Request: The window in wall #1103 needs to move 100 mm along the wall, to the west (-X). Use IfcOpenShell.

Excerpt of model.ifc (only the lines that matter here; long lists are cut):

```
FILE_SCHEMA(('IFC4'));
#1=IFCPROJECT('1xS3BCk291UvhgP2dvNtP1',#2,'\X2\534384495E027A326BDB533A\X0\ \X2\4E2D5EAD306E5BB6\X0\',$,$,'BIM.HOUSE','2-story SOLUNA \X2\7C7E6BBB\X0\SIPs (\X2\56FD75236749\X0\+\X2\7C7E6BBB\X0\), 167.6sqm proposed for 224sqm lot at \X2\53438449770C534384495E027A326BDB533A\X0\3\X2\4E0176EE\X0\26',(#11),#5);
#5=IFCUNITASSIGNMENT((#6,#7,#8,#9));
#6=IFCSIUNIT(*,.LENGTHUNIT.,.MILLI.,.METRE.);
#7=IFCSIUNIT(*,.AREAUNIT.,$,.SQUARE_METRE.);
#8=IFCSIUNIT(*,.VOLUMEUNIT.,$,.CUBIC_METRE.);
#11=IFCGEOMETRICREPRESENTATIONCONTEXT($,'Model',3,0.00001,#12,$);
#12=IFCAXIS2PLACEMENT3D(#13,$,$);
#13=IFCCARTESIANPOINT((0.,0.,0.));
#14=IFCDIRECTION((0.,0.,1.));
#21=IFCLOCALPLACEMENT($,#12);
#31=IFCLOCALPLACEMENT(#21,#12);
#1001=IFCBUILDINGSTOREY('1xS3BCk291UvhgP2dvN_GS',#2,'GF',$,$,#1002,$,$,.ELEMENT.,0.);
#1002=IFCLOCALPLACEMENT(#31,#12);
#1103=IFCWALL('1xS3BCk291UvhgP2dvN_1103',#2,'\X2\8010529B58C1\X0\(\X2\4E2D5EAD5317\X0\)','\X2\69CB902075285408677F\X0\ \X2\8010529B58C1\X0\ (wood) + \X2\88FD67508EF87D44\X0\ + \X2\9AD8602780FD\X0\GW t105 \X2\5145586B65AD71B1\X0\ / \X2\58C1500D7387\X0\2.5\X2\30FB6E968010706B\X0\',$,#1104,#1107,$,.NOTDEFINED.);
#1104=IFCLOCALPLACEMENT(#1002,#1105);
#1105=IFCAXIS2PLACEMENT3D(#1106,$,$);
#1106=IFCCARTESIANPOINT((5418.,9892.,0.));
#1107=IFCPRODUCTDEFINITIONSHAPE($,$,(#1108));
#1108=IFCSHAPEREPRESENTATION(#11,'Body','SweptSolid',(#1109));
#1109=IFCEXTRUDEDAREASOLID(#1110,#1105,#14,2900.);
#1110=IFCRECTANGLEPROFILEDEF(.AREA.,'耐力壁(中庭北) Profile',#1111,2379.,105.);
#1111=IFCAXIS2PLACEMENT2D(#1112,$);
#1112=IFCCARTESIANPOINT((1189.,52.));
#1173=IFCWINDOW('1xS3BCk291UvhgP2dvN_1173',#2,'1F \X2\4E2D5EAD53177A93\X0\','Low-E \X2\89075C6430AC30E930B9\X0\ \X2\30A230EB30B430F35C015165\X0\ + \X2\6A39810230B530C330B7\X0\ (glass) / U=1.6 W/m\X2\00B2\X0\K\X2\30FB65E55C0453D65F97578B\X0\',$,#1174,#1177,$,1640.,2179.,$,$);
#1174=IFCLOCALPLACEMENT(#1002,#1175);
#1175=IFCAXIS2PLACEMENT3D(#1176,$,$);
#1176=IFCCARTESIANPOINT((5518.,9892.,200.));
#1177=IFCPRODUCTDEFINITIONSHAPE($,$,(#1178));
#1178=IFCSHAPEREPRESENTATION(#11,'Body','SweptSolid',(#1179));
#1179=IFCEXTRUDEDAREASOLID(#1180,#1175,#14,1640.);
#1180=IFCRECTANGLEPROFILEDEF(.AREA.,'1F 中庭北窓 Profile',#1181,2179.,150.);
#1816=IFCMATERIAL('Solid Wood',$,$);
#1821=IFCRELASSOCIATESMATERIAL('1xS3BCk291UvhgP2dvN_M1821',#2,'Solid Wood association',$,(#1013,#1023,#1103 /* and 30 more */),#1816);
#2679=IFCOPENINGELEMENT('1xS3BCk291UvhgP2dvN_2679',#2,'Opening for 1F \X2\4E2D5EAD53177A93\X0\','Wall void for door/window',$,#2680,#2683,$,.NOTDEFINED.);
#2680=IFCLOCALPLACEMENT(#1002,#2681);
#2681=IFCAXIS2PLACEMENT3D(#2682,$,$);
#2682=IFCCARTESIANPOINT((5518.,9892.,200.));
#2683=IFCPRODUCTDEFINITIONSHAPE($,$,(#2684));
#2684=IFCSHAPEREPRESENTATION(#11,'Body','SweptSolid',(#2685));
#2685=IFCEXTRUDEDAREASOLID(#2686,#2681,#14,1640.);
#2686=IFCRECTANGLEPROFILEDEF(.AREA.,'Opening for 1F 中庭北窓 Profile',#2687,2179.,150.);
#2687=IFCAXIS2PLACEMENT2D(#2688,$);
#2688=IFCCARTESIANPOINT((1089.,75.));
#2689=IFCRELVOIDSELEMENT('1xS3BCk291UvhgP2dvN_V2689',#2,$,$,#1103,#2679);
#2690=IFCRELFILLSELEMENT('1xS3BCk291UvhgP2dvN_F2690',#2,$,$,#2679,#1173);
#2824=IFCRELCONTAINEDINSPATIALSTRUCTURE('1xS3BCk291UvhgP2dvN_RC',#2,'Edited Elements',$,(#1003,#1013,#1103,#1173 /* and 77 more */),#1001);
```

```python
import ifcopenshell
import ifcopenshell.api.geometry
import ifcopenshell.util.placement
import ifcopenshell.util.unit

model = ifcopenshell.open("model.ifc")
unit_scale = ifcopenshell.util.unit.calculate_unit_scale(model)

window = model.by_guid("1xS3BCk291UvhgP2dvN_1173")
opening = window.FillsVoids[0].RelatingOpeningElement
wall = opening.VoidsElements[0].RelatingBuildingElement

wall_matrix = ifcopenshell.util.placement.get_local_placement(wall.ObjectPlacement)
shift = wall_matrix[:3, 0] * -0.1 / unit_scale
before = ifcopenshell.util.placement.get_local_placement(window.ObjectPlacement)[:3, 3].copy()

# The window is not placed relative to its opening, so move both.
for product in (opening, window):
    matrix = ifcopenshell.util.placement.get_local_placement(product.ObjectPlacement)
    matrix[:3, 3] += shift
    ifcopenshell.api.geometry.edit_object_placement(model, product=product, matrix=matrix, is_si=False)

after = ifcopenshell.util.placement.get_local_placement(window.ObjectPlacement)[:3, 3]
print("window moved by", (after - before).round(3) + 0.0)

model.write("model_rev.ifc")
```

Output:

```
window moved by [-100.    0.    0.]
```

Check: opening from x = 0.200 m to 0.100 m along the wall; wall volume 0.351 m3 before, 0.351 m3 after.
